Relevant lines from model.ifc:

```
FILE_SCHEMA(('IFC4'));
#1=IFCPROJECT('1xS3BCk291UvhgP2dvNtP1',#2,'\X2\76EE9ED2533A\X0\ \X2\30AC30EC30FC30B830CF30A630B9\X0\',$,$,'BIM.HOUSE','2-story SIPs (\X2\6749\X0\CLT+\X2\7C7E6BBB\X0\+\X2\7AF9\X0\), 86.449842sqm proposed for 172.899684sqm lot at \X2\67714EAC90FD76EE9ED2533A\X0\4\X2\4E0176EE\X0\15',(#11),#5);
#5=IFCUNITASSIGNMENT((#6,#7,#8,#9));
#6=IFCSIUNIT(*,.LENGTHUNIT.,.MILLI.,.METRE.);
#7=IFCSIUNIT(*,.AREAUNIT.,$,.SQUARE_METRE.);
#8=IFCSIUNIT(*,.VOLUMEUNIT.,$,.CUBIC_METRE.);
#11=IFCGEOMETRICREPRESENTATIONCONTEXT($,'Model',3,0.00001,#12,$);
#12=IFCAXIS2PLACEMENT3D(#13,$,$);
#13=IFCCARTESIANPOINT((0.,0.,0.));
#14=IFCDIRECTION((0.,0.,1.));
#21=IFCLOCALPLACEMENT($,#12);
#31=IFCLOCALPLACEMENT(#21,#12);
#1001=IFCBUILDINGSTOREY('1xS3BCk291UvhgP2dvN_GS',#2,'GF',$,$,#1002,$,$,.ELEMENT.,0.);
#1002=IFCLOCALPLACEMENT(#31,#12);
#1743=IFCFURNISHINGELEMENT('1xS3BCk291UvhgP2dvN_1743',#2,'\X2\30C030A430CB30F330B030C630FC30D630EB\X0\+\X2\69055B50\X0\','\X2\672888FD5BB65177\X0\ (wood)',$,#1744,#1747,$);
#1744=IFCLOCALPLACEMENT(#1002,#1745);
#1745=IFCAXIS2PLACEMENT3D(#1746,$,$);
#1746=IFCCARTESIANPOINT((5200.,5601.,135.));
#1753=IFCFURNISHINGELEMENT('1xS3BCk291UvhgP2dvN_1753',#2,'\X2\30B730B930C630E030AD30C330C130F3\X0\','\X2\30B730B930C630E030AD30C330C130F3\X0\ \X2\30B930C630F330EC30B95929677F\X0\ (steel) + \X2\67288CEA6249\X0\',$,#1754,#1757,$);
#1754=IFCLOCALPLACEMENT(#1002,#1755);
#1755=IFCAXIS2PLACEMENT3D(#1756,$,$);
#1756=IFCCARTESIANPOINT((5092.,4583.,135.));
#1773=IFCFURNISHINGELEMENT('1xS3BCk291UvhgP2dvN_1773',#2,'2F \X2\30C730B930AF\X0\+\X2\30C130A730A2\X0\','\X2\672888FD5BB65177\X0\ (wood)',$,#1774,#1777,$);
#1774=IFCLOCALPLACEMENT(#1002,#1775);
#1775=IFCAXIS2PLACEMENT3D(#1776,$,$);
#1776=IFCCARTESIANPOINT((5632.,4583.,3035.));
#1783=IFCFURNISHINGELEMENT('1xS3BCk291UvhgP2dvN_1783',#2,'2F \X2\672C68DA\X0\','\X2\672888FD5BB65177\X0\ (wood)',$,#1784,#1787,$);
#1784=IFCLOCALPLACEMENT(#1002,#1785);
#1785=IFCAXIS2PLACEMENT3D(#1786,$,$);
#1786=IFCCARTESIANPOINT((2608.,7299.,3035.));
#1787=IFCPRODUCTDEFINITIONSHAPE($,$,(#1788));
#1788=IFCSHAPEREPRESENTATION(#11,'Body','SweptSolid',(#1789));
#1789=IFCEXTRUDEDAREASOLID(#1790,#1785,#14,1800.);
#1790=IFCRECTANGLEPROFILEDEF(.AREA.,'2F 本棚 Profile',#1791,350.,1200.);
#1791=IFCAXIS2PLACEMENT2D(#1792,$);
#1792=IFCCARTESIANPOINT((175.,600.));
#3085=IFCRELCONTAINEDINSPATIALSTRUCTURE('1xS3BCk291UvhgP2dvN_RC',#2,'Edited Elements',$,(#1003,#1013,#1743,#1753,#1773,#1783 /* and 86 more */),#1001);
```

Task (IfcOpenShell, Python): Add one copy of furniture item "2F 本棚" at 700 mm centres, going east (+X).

```python
import numpy as np
import ifcopenshell
import ifcopenshell.api.geometry
import ifcopenshell.api.root
import ifcopenshell.util.element
import ifcopenshell.util.placement
import ifcopenshell.util.unit

model = ifcopenshell.open("model.ifc")
unit_scale = ifcopenshell.util.unit.calculate_unit_scale(model)


def reuse_history(source, copy):
    """copy_class also copies each property set's owner history, people and application; keep the originals."""
    for rel in copy.IsDefinedBy:
        if rel.is_a("IfcRelDefinesByProperties") and (history := rel.RelatingPropertyDefinition.OwnerHistory):
            rel.RelatingPropertyDefinition.OwnerHistory = source.OwnerHistory
            ifcopenshell.util.element.remove_deep2(model, history)


source = model.by_guid("1xS3BCk291UvhgP2dvN_1783")
base = ifcopenshell.util.placement.get_local_placement(source.ObjectPlacement)
step = np.array([1.0, 0.0, 0.0]) * 0.7 / unit_scale

for i in range(1, 2):
    copy = ifcopenshell.api.root.copy_class(model, product=source)
    copy.Representation = ifcopenshell.util.element.copy_deep(
        model, source.Representation, exclude=["IfcGeometricRepresentationContext", "IfcRepresentationMap"]
    )
    reuse_history(source, copy)
    matrix = base.copy()
    matrix[:3, 3] += i * step
    print("added at", matrix[:3, 3].round(3) + 0.0)
    ifcopenshell.api.geometry.edit_object_placement(model, product=copy, matrix=matrix, is_si=False)

model.write("model_rev.ifc")
```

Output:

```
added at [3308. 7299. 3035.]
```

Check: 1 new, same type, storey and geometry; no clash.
